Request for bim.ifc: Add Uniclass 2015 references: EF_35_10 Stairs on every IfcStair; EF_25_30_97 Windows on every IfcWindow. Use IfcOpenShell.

First a look at what the model holds.

```python
import ifcopenshell

model = ifcopenshell.open("bim.ifc")
print(model.schema)
print("classifications:", [c.Name for c in model.by_type("IfcClassification")])
for ifc_class in ("IfcDoor", "IfcRoof", "IfcStair", "IfcWall", "IfcWindow"):
    print(ifc_class, len(model.by_type(ifc_class)))
```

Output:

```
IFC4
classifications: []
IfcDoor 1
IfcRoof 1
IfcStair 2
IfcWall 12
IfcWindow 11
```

```python
import ifcopenshell
import ifcopenshell.api.classification

model = ifcopenshell.open("bim.ifc")

system = ifcopenshell.api.classification.add_classification(model, classification="Uniclass 2015")

codes = {
    "IfcStair": ("EF_35_10", "Stairs"),
    "IfcWindow": ("EF_25_30_97", "Windows"),
}
for ifc_class, (code, name) in codes.items():
    products = model.by_type(ifc_class)
    ifcopenshell.api.classification.add_reference(
        model, products=products, classification=system, identification=code, name=name
    )
    print(code, len(products))

model.write("bim-out.ifc")
```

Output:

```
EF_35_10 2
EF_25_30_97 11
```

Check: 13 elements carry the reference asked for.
